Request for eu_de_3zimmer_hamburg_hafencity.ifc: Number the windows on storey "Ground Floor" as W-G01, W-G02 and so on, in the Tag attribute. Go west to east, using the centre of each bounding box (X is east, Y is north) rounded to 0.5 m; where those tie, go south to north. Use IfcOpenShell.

First a look at what the model holds.

```python
import ifcopenshell
import ifcopenshell.util.element
import ifcopenshell.util.placement

model = ifcopenshell.open("eu_de_3zimmer_hamburg_hafencity.ifc")
print(model.schema)
storey = next(s for s in model.by_type("IfcBuildingStorey") if s.Name == "Ground Floor")
windows = [e for e in ifcopenshell.util.element.get_decomposition(storey) if e.is_a("IfcWindow")]
for e in sorted(windows, key=lambda e: e.id()):
    origin = ifcopenshell.util.placement.get_local_placement(e.ObjectPlacement)[:3, 3]
    print(e.id(), e.Tag, e.Name, origin.round(2) + 0.0, sep=" | ")
```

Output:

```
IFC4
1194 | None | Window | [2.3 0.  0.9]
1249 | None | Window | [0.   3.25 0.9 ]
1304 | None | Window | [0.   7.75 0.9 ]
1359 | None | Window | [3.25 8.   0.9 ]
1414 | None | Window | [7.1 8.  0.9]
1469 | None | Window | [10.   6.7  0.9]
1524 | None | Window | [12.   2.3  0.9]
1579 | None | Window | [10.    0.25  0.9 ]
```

```python
import ifcopenshell
import ifcopenshell.geom
import ifcopenshell.util.element
import ifcopenshell.util.shape

model = ifcopenshell.open("eu_de_3zimmer_hamburg_hafencity.ifc")
settings = ifcopenshell.geom.settings()
settings.set("use-world-coords", True)


def centre(element):
    shape = ifcopenshell.geom.create_shape(settings, element)
    return ifcopenshell.util.shape.get_bbox_centroid(shape.geometry)


storey = next(s for s in model.by_type("IfcBuildingStorey") if s.Name == "Ground Floor")
windows = [e for e in ifcopenshell.util.element.get_decomposition(storey) if e.is_a("IfcWindow")]

# Insertion points can sit at a corner or the storey origin, so sort by the geometry (in metres).
centres = {e: centre(e) for e in windows}
windows.sort(key=lambda e: (round(centres[e][0] / 0.5), centres[e][1]))

for i, e in enumerate(windows, start=1):
    number = f"W-G{i:02d}"
    e.Tag = number
    print(e.id(), number)

model.write("eu_de_3zimmer_hamburg_hafencity_rev.ifc")
```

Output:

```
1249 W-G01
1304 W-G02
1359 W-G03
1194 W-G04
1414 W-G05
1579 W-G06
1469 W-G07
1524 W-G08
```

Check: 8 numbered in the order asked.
